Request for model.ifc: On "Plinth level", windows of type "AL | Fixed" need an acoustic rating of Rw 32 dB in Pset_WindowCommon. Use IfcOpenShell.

First a look at what the model holds.

```python
import ifcopenshell
import ifcopenshell.util.element

model = ifcopenshell.open("model.ifc")
print(model.schema)
storey = next(s for s in model.by_type("IfcBuildingStorey") if s.Name == "Plinth level")
windows = [e for e in ifcopenshell.util.element.get_decomposition(storey) if e.is_a("IfcWindow")]
seen = {}
for e in windows:
    element_type = ifcopenshell.util.element.get_type(e)
    key = (element_type.Name if element_type != e and element_type else None, ifcopenshell.util.element.get_pset(e, "Pset_WindowCommon", "AcousticRating"))
    seen[key] = seen.get(key, 0) + 1
for (name, value), count in sorted(seen.items(), key=str):
    print(count, "x", name, "|", value)
```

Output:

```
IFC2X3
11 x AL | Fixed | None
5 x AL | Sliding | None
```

```python
import ifcopenshell
import ifcopenshell.api.pset
import ifcopenshell.util.element

model = ifcopenshell.open("model.ifc")

storey = next(s for s in model.by_type("IfcBuildingStorey") if s.Name == "Plinth level")
windows = [e for e in ifcopenshell.util.element.get_decomposition(storey) if e.is_a("IfcWindow")]

count = 0
for e in windows:
    element_type = ifcopenshell.util.element.get_type(e)
    if element_type in (None, e) or element_type.Name != "AL | Fixed":
        continue
    # add_pset returns the element's existing set when there is one.
    pset = ifcopenshell.api.pset.add_pset(model, product=e, name="Pset_WindowCommon")
    ifcopenshell.api.pset.edit_pset(model, pset=pset, properties={"AcousticRating": "Rw 32 dB"})
    count += 1

print(count, "windows updated")

model.write("model_updated.ifc")
```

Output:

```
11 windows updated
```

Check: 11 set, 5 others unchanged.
